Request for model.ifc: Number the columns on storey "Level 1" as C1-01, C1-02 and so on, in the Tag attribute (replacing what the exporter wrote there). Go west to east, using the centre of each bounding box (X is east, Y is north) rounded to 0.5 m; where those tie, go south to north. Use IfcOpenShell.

First a look at what the model holds.

```python
import ifcopenshell
import ifcopenshell.util.element
import ifcopenshell.util.placement

model = ifcopenshell.open("model.ifc")
print(model.schema)
storey = next(s for s in model.by_type("IfcBuildingStorey") if s.Name == "Level 1")
columns = [e for e in ifcopenshell.util.element.get_decomposition(storey) if e.is_a("IfcColumn")]
for e in sorted(columns, key=lambda e: e.id()):
    origin = ifcopenshell.util.placement.get_local_placement(e.ObjectPlacement)[:3, 3]
    print(e.id(), e.Tag, e.Name, origin.round(2) + 0.0, sep=" | ")
```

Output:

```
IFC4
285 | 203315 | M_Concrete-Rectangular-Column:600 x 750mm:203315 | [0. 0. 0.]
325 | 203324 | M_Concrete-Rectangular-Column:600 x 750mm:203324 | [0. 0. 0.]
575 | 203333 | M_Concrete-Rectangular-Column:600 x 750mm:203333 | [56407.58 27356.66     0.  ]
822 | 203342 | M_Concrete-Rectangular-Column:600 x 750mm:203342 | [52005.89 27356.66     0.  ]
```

```python
import ifcopenshell
import ifcopenshell.geom
import ifcopenshell.util.element
import ifcopenshell.util.shape

model = ifcopenshell.open("model.ifc")
settings = ifcopenshell.geom.settings()
settings.set("use-world-coords", True)


def centre(element):
    shape = ifcopenshell.geom.create_shape(settings, element)
    return ifcopenshell.util.shape.get_bbox_centroid(shape.geometry)


storey = next(s for s in model.by_type("IfcBuildingStorey") if s.Name == "Level 1")
columns = [e for e in ifcopenshell.util.element.get_decomposition(storey) if e.is_a("IfcColumn")]

# Insertion points can sit at a corner or the storey origin, so sort by the geometry (in metres).
centres = {e: centre(e) for e in columns}
columns.sort(key=lambda e: (round(centres[e][0] / 0.5), centres[e][1]))

for i, e in enumerate(columns, start=1):
    number = f"C1-{i:02d}"
    e.Tag = number
    print(e.id(), number)

model.write("model_updated.ifc")
```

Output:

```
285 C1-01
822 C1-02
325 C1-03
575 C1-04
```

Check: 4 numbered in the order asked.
